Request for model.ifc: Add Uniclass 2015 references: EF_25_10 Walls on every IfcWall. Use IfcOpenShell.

First a look at what the model holds.

```python
import ifcopenshell

model = ifcopenshell.open("model.ifc")
print(model.schema)
print("classifications:", [c.Name for c in model.by_type("IfcClassification")])
for ifc_class in ("IfcDoor", "IfcRoof", "IfcStair", "IfcWall", "IfcWindow"):
    print(ifc_class, len(model.by_type(ifc_class)))
```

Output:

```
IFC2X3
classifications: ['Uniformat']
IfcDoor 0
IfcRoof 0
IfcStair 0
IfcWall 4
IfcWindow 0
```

```python
import ifcopenshell
import ifcopenshell.api.classification

model = ifcopenshell.open("model.ifc")

# IFC2X3 requires Source and Edition and has no link from the project to the system.
system = model.create_entity("IfcClassification", Source="NBS", Edition="2015", Name="Uniclass 2015")

codes = {
    "IfcWall": ("EF_25_10", "Walls"),
}
for ifc_class, (code, name) in codes.items():
    products = model.by_type(ifc_class)
    ifcopenshell.api.classification.add_reference(
        model, products=products, classification=system, identification=code, name=name
    )
    print(code, len(products))

model.write("model_edited.ifc")
```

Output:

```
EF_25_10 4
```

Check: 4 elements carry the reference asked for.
